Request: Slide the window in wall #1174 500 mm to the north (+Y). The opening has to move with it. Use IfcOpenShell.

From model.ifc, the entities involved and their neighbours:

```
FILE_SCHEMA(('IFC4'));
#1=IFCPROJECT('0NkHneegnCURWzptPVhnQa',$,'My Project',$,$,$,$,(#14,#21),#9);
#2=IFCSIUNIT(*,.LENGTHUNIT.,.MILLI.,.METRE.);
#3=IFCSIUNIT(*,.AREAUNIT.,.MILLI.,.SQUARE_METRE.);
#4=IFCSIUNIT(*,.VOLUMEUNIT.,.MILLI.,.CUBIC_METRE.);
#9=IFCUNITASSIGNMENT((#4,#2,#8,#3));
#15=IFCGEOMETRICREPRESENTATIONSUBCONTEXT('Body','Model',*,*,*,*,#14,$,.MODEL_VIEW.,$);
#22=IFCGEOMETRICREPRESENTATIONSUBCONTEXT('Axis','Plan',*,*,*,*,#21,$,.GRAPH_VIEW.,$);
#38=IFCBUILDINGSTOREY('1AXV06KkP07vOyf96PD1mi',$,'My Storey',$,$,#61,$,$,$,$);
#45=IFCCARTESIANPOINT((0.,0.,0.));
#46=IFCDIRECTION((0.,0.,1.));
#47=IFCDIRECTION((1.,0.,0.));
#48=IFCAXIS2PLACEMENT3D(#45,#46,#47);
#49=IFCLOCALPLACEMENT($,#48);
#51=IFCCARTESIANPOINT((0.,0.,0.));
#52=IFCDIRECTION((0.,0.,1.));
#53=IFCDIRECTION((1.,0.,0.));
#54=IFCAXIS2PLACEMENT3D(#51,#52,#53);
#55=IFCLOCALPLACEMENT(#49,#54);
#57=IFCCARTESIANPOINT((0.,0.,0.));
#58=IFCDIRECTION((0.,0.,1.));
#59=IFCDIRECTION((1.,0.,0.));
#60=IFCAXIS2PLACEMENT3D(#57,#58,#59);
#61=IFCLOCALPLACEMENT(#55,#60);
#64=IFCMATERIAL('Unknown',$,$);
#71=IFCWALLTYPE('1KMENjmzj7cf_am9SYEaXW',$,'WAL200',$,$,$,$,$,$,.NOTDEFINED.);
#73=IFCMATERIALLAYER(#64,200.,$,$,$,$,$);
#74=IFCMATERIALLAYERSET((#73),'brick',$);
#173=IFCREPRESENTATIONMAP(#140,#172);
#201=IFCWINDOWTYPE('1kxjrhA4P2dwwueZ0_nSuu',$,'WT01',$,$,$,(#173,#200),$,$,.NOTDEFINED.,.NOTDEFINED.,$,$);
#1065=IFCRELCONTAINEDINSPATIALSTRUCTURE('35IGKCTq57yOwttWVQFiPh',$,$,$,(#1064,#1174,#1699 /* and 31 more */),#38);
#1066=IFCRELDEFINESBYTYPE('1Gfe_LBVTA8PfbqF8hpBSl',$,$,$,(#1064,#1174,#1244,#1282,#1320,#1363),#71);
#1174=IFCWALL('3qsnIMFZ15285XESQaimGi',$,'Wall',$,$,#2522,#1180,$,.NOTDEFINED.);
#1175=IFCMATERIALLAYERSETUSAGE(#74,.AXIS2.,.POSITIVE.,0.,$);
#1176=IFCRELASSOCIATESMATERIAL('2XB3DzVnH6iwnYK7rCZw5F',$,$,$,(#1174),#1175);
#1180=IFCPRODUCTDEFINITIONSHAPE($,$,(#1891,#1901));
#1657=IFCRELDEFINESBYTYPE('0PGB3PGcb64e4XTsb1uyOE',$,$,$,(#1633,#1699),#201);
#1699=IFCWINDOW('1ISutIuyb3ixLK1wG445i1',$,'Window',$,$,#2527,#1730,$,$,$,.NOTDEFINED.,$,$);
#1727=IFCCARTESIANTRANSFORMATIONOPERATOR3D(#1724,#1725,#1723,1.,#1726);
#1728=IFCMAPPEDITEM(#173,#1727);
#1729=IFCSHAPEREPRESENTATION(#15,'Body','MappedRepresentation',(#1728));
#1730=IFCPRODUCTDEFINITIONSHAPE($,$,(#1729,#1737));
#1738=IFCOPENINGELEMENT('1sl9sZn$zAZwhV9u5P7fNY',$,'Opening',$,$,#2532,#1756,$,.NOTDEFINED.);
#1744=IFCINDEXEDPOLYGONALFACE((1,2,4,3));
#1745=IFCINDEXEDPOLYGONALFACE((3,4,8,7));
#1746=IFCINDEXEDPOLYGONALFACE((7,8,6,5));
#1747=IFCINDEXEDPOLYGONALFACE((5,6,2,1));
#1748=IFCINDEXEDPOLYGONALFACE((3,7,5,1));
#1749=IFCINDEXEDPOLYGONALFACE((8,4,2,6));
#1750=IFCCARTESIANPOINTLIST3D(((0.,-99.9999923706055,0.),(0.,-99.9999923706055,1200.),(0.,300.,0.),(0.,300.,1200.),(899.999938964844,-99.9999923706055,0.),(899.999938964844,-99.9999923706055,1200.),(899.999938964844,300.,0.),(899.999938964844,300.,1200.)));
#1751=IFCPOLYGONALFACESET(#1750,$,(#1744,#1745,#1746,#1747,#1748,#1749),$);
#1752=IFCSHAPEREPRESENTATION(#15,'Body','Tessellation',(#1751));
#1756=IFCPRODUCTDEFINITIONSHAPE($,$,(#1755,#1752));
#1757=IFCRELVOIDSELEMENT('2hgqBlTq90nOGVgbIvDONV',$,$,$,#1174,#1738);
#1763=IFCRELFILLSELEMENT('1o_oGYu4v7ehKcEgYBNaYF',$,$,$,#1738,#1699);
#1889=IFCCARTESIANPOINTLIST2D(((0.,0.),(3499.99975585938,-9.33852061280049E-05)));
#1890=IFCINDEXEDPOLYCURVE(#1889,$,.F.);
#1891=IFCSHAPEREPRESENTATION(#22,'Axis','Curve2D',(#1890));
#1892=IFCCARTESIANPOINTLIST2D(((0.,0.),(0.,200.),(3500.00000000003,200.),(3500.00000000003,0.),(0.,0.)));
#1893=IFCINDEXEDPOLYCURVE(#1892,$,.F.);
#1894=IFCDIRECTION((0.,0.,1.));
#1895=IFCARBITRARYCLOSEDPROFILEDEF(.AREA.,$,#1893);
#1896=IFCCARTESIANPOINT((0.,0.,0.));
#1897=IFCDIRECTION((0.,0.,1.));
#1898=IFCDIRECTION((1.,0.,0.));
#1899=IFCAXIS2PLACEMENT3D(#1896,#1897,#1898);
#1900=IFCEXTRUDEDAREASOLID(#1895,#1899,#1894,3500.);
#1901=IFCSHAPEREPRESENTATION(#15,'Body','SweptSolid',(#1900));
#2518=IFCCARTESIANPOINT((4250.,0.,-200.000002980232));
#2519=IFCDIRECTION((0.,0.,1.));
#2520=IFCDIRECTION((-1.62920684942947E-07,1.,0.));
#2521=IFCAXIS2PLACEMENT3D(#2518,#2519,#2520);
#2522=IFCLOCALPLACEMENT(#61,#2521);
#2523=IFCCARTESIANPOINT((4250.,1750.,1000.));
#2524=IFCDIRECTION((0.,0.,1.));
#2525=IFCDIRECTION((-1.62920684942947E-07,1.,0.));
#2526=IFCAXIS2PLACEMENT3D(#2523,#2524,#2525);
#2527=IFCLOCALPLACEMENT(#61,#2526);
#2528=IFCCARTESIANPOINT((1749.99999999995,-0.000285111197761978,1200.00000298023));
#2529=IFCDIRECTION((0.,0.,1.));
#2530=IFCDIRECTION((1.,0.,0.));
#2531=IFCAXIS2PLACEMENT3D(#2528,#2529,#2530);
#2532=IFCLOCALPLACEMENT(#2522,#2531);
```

```python
import ifcopenshell
import ifcopenshell.api.geometry
import ifcopenshell.util.placement
import ifcopenshell.util.unit

model = ifcopenshell.open("model.ifc")
unit_scale = ifcopenshell.util.unit.calculate_unit_scale(model)

window = model.by_guid("1ISutIuyb3ixLK1wG445i1")
opening = window.FillsVoids[0].RelatingOpeningElement
wall = opening.VoidsElements[0].RelatingBuildingElement

wall_matrix = ifcopenshell.util.placement.get_local_placement(wall.ObjectPlacement)
shift = wall_matrix[:3, 0] * 0.5 / unit_scale
before = ifcopenshell.util.placement.get_local_placement(window.ObjectPlacement)[:3, 3].copy()

# The window is not placed relative to its opening, so move both.
for product in (opening, window):
    matrix = ifcopenshell.util.placement.get_local_placement(product.ObjectPlacement)
    matrix[:3, 3] += shift
    ifcopenshell.api.geometry.edit_object_placement(model, product=product, matrix=matrix, is_si=False)

after = ifcopenshell.util.placement.get_local_placement(window.ObjectPlacement)[:3, 3]
print("window moved by", (after - before).round(3) + 0.0)

model.write("model-out.ifc")
```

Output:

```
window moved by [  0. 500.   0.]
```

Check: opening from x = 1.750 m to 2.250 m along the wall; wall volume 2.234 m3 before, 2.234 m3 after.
